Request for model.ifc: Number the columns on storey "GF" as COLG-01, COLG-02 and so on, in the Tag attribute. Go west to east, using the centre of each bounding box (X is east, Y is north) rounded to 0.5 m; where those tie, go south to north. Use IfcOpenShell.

First a look at what the model holds.

```python
import ifcopenshell
import ifcopenshell.util.element
import ifcopenshell.util.placement

model = ifcopenshell.open("model.ifc")
print(model.schema)
storey = next(s for s in model.by_type("IfcBuildingStorey") if s.Name == "GF")
columns = [e for e in ifcopenshell.util.element.get_decomposition(storey) if e.is_a("IfcColumn")]
for e in sorted(columns, key=lambda e: e.id()):
    origin = ifcopenshell.util.placement.get_local_placement(e.ObjectPlacement)[:3, 3]
    print(e.id(), e.Tag, e.Name, origin.round(2) + 0.0, sep=" | ")
```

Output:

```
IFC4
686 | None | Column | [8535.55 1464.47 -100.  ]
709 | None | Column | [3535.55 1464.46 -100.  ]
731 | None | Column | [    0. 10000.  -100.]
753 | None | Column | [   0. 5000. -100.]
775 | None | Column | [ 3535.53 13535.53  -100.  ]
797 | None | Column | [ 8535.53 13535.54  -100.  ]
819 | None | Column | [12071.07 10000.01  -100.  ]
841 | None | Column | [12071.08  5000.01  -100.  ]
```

```python
import ifcopenshell
import ifcopenshell.geom
import ifcopenshell.util.element
import ifcopenshell.util.shape

model = ifcopenshell.open("model.ifc")
settings = ifcopenshell.geom.settings()
settings.set("use-world-coords", True)


def centre(element):
    shape = ifcopenshell.geom.create_shape(settings, element)
    return ifcopenshell.util.shape.get_bbox_centroid(shape.geometry)


storey = next(s for s in model.by_type("IfcBuildingStorey") if s.Name == "GF")
columns = [e for e in ifcopenshell.util.element.get_decomposition(storey) if e.is_a("IfcColumn")]

# Insertion points can sit at a corner or the storey origin, so sort by the geometry (in metres).
centres = {e: centre(e) for e in columns}
columns.sort(key=lambda e: (round(centres[e][0] / 0.5), centres[e][1]))

for i, e in enumerate(columns, start=1):
    number = f"COLG-{i:02d}"
    e.Tag = number
    print(e.id(), number)

model.write("model_rev.ifc")
```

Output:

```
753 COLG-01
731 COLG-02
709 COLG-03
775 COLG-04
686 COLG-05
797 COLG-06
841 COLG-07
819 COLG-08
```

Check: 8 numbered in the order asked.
